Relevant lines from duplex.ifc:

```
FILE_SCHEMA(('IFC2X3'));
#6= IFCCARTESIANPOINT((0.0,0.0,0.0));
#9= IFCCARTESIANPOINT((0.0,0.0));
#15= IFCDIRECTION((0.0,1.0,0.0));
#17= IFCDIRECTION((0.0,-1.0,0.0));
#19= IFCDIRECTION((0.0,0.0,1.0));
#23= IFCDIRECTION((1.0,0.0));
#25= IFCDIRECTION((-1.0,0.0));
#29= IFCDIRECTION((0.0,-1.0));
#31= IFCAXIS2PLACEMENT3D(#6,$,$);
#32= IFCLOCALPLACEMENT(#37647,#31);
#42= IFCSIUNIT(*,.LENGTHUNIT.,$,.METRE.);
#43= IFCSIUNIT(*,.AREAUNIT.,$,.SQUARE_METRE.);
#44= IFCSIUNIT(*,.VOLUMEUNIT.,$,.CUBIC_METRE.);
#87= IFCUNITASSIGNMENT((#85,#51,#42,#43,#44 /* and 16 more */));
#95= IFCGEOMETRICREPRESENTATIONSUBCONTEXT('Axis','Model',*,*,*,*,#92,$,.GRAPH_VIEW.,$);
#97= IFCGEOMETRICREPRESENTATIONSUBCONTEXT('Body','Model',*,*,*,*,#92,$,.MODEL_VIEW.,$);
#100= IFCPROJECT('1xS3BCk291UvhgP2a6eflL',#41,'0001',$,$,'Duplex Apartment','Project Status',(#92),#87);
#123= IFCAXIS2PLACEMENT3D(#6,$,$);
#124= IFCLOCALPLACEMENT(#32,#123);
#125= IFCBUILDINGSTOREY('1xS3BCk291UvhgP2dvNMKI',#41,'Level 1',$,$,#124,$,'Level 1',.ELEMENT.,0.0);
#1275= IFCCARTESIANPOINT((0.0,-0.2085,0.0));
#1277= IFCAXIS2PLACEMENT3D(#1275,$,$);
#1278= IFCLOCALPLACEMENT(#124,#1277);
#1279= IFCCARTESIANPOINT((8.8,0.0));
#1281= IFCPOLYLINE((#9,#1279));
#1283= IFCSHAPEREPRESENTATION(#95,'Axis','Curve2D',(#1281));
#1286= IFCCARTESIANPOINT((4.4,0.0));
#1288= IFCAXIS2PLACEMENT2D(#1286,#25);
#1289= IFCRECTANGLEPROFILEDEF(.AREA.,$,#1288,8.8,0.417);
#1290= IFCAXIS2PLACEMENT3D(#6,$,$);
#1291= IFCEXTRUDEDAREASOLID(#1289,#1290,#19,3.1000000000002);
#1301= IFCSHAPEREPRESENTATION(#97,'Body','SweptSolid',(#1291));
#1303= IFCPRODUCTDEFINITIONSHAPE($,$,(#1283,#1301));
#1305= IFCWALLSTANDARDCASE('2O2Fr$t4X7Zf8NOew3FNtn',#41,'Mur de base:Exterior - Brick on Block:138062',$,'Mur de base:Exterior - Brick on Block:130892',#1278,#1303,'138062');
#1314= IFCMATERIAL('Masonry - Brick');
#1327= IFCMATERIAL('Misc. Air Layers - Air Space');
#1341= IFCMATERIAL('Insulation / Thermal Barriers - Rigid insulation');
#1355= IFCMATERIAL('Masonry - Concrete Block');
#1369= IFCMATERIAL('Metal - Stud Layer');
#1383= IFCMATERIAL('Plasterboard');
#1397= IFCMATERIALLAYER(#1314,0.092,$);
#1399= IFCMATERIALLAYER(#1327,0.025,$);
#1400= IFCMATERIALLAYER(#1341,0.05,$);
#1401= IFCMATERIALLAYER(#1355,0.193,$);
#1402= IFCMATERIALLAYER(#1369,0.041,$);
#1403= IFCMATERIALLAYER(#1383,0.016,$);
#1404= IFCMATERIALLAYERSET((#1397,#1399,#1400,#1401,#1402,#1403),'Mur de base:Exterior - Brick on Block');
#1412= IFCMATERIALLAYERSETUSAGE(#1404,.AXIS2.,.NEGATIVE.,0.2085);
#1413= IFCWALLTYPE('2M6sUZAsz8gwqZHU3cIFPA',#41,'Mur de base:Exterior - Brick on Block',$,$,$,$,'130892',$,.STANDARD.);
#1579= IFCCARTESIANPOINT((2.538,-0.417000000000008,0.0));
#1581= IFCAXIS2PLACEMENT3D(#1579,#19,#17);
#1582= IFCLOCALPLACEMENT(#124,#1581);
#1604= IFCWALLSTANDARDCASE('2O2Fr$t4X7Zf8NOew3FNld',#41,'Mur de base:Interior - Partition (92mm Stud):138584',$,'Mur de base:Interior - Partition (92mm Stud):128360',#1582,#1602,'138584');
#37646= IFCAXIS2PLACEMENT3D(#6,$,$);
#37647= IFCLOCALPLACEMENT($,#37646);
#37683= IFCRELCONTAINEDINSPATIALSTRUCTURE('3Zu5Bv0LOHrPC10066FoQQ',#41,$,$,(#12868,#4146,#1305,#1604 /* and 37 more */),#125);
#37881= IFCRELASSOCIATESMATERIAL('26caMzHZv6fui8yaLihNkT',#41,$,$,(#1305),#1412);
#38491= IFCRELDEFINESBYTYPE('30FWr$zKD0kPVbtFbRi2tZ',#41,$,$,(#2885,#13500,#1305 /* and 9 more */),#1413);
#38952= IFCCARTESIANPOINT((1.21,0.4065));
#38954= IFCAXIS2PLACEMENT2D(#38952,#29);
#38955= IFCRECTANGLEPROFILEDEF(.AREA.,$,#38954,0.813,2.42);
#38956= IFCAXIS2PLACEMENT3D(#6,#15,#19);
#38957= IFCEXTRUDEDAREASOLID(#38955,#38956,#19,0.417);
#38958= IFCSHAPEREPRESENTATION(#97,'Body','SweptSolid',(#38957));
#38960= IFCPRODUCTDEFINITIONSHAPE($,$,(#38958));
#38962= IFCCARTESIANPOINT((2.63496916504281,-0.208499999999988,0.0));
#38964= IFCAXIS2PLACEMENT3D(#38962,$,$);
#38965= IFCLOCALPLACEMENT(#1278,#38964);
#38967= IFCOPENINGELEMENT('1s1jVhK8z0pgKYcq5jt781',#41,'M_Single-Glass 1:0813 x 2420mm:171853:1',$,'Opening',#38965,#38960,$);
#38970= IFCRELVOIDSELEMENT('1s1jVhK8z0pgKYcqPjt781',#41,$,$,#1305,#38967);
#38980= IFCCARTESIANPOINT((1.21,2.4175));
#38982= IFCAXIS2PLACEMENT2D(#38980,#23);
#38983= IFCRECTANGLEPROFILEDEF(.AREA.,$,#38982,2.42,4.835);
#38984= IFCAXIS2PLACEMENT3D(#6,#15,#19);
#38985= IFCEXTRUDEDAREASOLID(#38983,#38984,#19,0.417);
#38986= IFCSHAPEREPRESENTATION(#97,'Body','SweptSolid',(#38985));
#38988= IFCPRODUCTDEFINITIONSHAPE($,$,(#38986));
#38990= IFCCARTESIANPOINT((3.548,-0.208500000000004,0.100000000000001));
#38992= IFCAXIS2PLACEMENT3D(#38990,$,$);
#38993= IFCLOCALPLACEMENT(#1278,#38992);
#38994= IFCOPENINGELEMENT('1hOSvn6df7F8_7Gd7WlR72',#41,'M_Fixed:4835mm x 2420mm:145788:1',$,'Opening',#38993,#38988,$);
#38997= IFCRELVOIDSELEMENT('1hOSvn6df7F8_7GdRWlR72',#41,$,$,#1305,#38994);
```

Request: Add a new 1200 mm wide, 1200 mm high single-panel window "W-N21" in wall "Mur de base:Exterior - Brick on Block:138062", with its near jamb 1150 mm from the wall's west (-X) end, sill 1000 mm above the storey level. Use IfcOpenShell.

```python
import numpy as np
import ifcopenshell
import ifcopenshell.api.feature
import ifcopenshell.api.geometry
import ifcopenshell.api.root
import ifcopenshell.api.spatial
import ifcopenshell.api.type
import ifcopenshell.geom
import ifcopenshell.util.element
import ifcopenshell.util.placement
import ifcopenshell.util.representation
import ifcopenshell.util.shape
import ifcopenshell.util.unit

model = ifcopenshell.open("duplex.ifc")
unit_scale = ifcopenshell.util.unit.calculate_unit_scale(model)
settings = ifcopenshell.geom.settings()


def volume(element):
    """Net volume in cubic metres, openings subtracted."""
    shape = ifcopenshell.geom.create_shape(settings, element)
    return ifcopenshell.util.shape.get_volume(shape.geometry)


wall = model.by_guid("2O2Fr$t4X7Zf8NOew3FNtn")
storey = ifcopenshell.util.element.get_container(wall, ifc_class="IfcBuildingStorey")
context = ifcopenshell.util.representation.get_context(model, "Model", "Body", "MODEL_VIEW")
before = volume(wall)

width, height, from_end, sill = 1.2, 1.2, 1.15, 1  # metres

# The wall runs along its own X axis, and the end named is its -X end.
wall_shape = ifcopenshell.geom.create_shape(settings, wall)
x, y, z = ifcopenshell.util.shape.get_vertices(wall_shape.geometry).T
start = x.min() + from_end
face, thickness = float(y.min()), float(y.max() - y.min())
wall_matrix = ifcopenshell.util.placement.get_local_placement(wall.ObjectPlacement)
level = ifcopenshell.util.placement.get_local_placement(storey.ObjectPlacement)[2, 3]


def in_wall(x, y):
    """Placement at x, y metres in the wall's axes, at sill height."""
    matrix = wall_matrix.copy()
    matrix[:, 3] = wall_matrix @ np.array([x / unit_scale, y / unit_scale, 0.0, 1.0])
    matrix[2, 3] = level + sill / unit_scale
    return matrix


# Opening: a box that overshoots both wall faces by 50 mm.
opening = ifcopenshell.api.root.create_entity(model, ifc_class="IfcOpeningElement")
box = ifcopenshell.api.geometry.add_wall_representation(
    model, context=context, length=width, height=height, thickness=thickness + 0.1
)
ifcopenshell.api.geometry.assign_representation(model, product=opening, representation=box)
ifcopenshell.api.geometry.edit_object_placement(model, product=opening, matrix=in_wall(start, face - 0.05), is_si=False)
ifcopenshell.api.feature.add_feature(model, feature=opening, element=wall)

window = ifcopenshell.api.root.create_entity(model, ifc_class="IfcWindow", name="W-N21")
window.OverallWidth, window.OverallHeight = width / unit_scale, height / unit_scale
body = ifcopenshell.api.geometry.add_window_representation(
    model,
    context=context,
    overall_width=window.OverallWidth,
    overall_height=window.OverallHeight,
    partition_type="SINGLE_PANEL",
)
ifcopenshell.api.geometry.assign_representation(model, product=window, representation=body)
ifcopenshell.api.spatial.assign_container(model, products=[window], relating_structure=storey)
fills = ifcopenshell.api.feature.add_filling(model, opening=opening, element=window)
fills.OwnerHistory = window.OwnerHistory  # required in IFC2X3

# IFC2X3 keeps the operation on the window style.
style = ifcopenshell.api.root.create_entity(model, ifc_class="IfcWindowStyle", name="W-N21")
style.OperationType, style.ConstructionType = "SINGLE_PANEL", "NOTDEFINED"
style.ParameterTakesPrecedence = style.Sizeable = False
ifcopenshell.api.type.assign_type(model, related_objects=[window], relating_type=style)

# Centre the window in the wall's thickness.
ifcopenshell.api.geometry.edit_object_placement(model, product=window, matrix=in_wall(start, face), is_si=False)
window_shape = ifcopenshell.geom.create_shape(settings, window)
depth = ifcopenshell.util.shape.get_vertices(window_shape.geometry)[:, 1]
offset = face + thickness / 2 - (depth.min() + depth.max()) / 2
ifcopenshell.api.geometry.edit_object_placement(model, product=window, matrix=in_wall(start, offset), is_si=False)

after = volume(wall)

print(f"wall volume {before:.3f} -> {after:.3f} m3")

model.write("duplex_rev.ifc")
```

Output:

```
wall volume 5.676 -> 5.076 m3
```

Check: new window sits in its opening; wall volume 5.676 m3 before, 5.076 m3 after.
